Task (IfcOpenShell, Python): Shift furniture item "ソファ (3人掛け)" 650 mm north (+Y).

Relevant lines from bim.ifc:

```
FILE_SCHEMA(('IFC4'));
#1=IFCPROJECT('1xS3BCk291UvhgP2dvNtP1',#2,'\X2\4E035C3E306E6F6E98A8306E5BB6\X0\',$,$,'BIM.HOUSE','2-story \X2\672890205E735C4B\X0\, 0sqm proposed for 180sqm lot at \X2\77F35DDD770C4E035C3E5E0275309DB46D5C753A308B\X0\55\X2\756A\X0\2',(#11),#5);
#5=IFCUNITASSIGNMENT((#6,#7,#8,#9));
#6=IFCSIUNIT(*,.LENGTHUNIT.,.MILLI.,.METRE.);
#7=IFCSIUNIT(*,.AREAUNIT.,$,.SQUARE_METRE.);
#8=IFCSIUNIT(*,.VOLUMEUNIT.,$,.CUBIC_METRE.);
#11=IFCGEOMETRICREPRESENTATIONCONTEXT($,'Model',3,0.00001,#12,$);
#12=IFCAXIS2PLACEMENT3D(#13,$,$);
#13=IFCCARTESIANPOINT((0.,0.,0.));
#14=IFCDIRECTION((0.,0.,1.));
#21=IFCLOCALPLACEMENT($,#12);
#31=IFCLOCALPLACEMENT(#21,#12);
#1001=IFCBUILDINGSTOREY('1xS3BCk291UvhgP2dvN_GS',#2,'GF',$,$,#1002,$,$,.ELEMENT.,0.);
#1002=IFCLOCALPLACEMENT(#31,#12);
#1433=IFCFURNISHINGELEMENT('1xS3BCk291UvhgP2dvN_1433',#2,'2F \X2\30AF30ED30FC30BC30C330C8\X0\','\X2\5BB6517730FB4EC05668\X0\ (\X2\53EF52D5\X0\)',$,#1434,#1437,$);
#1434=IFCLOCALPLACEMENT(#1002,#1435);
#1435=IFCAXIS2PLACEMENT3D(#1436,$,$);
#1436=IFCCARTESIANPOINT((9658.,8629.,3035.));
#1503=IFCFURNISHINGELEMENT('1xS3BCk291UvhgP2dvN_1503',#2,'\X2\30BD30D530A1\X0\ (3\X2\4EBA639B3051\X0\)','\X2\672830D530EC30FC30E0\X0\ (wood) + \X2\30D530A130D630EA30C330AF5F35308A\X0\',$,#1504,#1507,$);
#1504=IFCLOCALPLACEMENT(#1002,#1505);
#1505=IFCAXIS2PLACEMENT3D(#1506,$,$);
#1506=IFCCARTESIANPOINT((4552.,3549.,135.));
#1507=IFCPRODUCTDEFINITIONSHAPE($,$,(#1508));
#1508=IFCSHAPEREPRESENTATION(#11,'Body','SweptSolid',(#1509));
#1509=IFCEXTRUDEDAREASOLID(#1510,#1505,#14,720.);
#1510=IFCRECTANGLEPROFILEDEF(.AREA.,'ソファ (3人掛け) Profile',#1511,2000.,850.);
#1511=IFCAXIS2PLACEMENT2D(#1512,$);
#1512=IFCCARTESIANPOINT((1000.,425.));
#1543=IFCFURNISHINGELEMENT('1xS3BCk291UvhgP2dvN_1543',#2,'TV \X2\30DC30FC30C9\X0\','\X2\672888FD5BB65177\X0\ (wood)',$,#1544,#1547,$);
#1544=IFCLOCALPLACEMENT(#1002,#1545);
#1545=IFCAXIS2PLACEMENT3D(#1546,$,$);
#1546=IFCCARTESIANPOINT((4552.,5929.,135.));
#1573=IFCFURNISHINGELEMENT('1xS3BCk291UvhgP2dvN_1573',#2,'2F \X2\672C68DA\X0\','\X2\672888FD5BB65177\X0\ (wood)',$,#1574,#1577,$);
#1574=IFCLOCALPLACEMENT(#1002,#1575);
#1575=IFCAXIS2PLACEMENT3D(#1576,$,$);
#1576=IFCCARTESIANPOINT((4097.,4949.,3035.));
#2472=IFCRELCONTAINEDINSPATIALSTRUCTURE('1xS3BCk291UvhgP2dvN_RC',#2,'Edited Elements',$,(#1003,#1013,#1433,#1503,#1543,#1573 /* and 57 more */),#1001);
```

```python
import ifcopenshell
import ifcopenshell.api.geometry
import ifcopenshell.util.placement
import ifcopenshell.util.unit

model = ifcopenshell.open("bim.ifc")
unit_scale = ifcopenshell.util.unit.calculate_unit_scale(model)

item = model.by_guid("1xS3BCk291UvhgP2dvN_1503")
matrix = ifcopenshell.util.placement.get_local_placement(item.ObjectPlacement)
matrix[1, 3] += 0.65 / unit_scale
ifcopenshell.api.geometry.edit_object_placement(model, product=item, matrix=matrix, is_si=False)

print(ifcopenshell.util.placement.get_local_placement(item.ObjectPlacement).round(3) + 0.0)

model.write("bim_updated.ifc")
```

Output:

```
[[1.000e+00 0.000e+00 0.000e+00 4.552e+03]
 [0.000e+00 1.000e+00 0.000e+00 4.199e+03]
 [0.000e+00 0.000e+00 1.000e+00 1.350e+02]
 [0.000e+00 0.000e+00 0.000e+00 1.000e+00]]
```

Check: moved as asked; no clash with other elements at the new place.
